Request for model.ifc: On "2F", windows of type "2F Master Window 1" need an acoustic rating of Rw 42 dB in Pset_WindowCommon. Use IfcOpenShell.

First a look at what the model holds.

```python
import ifcopenshell
import ifcopenshell.util.element

model = ifcopenshell.open("model.ifc")
print(model.schema)
storey = next(s for s in model.by_type("IfcBuildingStorey") if s.Name == "2F")
windows = [e for e in ifcopenshell.util.element.get_decomposition(storey) if e.is_a("IfcWindow")]
seen = {}
for e in windows:
    element_type = ifcopenshell.util.element.get_type(e)
    key = (element_type.Name if element_type != e and element_type else None, ifcopenshell.util.element.get_pset(e, "Pset_WindowCommon", "AcousticRating"))
    seen[key] = seen.get(key, 0) + 1
for (name, value), count in sorted(seen.items(), key=str):
    print(count, "x", name, "|", value)
```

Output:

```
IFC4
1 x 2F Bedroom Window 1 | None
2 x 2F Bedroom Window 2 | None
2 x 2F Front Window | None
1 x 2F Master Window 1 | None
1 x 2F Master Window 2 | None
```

```python
import ifcopenshell
import ifcopenshell.api.pset
import ifcopenshell.util.element

model = ifcopenshell.open("model.ifc")

storey = next(s for s in model.by_type("IfcBuildingStorey") if s.Name == "2F")
windows = [e for e in ifcopenshell.util.element.get_decomposition(storey) if e.is_a("IfcWindow")]

count = 0
for e in windows:
    element_type = ifcopenshell.util.element.get_type(e)
    if element_type in (None, e) or element_type.Name != "2F Master Window 1":
        continue
    # add_pset returns the element's existing set when there is one.
    pset = ifcopenshell.api.pset.add_pset(model, product=e, name="Pset_WindowCommon")
    ifcopenshell.api.pset.edit_pset(model, pset=pset, properties={"AcousticRating": "Rw 42 dB"})
    count += 1

print(count, "windows updated")

model.write("model_rev.ifc")
```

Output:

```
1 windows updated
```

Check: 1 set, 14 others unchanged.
